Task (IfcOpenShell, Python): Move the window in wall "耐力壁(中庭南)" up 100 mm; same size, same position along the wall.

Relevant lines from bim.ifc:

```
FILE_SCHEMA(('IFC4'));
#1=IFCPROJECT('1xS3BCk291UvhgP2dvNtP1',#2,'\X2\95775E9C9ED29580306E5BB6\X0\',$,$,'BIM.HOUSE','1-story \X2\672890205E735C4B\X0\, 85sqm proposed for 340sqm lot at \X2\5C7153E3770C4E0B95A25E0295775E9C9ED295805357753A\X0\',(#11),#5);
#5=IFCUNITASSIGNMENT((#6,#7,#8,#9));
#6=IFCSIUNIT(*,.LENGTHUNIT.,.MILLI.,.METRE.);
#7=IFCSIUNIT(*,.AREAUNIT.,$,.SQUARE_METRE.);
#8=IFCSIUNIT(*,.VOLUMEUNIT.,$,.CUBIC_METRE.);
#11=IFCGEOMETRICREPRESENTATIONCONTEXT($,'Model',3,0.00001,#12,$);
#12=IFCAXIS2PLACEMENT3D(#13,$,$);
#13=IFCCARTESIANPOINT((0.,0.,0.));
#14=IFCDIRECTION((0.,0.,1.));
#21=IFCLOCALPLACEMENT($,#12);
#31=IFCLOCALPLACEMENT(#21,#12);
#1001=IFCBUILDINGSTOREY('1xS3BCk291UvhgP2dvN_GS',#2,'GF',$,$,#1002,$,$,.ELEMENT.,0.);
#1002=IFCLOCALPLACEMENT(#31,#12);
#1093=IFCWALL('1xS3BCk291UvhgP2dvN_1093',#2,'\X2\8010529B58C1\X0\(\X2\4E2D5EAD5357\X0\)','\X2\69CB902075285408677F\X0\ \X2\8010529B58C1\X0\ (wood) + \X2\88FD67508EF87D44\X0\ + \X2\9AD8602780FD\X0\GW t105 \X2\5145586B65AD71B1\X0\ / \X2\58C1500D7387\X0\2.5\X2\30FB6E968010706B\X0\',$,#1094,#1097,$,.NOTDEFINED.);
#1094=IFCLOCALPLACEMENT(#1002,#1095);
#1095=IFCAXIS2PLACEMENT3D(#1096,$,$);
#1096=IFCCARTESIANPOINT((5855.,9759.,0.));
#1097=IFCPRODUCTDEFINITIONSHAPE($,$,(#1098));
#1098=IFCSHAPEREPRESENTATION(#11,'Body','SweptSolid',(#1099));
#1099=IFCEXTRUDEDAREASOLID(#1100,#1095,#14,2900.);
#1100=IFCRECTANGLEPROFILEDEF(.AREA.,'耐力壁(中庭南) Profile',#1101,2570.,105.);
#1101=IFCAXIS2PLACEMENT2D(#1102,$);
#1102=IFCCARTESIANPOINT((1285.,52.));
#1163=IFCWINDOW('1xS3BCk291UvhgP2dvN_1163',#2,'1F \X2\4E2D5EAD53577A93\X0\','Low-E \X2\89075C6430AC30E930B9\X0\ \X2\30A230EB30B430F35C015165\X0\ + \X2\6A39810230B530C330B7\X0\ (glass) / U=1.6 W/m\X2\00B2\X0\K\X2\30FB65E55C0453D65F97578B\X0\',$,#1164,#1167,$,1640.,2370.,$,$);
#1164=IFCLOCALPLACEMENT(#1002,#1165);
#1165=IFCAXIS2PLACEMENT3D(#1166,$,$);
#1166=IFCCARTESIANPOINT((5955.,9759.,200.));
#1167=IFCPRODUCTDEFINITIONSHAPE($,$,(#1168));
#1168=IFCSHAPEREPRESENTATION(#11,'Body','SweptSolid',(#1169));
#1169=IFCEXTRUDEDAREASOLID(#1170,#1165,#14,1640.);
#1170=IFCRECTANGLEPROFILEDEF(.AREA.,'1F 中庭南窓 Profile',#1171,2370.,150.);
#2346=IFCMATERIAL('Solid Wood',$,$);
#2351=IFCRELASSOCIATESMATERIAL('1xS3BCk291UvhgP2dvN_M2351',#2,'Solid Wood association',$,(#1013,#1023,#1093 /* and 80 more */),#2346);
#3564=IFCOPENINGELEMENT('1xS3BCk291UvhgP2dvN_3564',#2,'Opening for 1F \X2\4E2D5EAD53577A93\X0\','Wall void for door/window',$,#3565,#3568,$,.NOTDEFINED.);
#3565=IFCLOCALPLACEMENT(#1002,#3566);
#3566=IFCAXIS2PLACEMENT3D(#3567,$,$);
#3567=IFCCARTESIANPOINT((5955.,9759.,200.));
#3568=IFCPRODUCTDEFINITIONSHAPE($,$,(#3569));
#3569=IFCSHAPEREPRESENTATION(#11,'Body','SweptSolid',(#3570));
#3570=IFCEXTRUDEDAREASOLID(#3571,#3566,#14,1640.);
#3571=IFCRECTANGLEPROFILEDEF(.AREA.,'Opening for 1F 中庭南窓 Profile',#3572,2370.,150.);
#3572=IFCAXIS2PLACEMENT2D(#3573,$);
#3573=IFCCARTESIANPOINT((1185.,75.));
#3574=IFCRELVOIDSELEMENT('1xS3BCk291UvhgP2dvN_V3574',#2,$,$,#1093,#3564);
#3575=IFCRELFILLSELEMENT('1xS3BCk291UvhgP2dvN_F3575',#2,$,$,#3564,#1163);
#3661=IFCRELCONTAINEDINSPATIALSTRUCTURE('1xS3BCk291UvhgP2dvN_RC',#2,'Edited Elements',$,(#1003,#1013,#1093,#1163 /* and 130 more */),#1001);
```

```python
import numpy as np
import ifcopenshell
import ifcopenshell.api.geometry
import ifcopenshell.util.placement
import ifcopenshell.util.unit

model = ifcopenshell.open("bim.ifc")
unit_scale = ifcopenshell.util.unit.calculate_unit_scale(model)

window = model.by_id(1163)
opening = window.FillsVoids[0].RelatingOpeningElement
dz = 0.1 / unit_scale

shift = np.array([0.0, 0.0, dz])
# The window is not placed relative to its opening, so move both.
for product in (opening, window):
    matrix = ifcopenshell.util.placement.get_local_placement(product.ObjectPlacement)
    matrix[:3, 3] += shift
    ifcopenshell.api.geometry.edit_object_placement(model, product=product, matrix=matrix, is_si=False)

print(f"moved by {dz * unit_scale:+.3f} m")

model.write("bim-out.ifc")
```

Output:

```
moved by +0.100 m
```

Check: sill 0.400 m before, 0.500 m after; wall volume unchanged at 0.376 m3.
